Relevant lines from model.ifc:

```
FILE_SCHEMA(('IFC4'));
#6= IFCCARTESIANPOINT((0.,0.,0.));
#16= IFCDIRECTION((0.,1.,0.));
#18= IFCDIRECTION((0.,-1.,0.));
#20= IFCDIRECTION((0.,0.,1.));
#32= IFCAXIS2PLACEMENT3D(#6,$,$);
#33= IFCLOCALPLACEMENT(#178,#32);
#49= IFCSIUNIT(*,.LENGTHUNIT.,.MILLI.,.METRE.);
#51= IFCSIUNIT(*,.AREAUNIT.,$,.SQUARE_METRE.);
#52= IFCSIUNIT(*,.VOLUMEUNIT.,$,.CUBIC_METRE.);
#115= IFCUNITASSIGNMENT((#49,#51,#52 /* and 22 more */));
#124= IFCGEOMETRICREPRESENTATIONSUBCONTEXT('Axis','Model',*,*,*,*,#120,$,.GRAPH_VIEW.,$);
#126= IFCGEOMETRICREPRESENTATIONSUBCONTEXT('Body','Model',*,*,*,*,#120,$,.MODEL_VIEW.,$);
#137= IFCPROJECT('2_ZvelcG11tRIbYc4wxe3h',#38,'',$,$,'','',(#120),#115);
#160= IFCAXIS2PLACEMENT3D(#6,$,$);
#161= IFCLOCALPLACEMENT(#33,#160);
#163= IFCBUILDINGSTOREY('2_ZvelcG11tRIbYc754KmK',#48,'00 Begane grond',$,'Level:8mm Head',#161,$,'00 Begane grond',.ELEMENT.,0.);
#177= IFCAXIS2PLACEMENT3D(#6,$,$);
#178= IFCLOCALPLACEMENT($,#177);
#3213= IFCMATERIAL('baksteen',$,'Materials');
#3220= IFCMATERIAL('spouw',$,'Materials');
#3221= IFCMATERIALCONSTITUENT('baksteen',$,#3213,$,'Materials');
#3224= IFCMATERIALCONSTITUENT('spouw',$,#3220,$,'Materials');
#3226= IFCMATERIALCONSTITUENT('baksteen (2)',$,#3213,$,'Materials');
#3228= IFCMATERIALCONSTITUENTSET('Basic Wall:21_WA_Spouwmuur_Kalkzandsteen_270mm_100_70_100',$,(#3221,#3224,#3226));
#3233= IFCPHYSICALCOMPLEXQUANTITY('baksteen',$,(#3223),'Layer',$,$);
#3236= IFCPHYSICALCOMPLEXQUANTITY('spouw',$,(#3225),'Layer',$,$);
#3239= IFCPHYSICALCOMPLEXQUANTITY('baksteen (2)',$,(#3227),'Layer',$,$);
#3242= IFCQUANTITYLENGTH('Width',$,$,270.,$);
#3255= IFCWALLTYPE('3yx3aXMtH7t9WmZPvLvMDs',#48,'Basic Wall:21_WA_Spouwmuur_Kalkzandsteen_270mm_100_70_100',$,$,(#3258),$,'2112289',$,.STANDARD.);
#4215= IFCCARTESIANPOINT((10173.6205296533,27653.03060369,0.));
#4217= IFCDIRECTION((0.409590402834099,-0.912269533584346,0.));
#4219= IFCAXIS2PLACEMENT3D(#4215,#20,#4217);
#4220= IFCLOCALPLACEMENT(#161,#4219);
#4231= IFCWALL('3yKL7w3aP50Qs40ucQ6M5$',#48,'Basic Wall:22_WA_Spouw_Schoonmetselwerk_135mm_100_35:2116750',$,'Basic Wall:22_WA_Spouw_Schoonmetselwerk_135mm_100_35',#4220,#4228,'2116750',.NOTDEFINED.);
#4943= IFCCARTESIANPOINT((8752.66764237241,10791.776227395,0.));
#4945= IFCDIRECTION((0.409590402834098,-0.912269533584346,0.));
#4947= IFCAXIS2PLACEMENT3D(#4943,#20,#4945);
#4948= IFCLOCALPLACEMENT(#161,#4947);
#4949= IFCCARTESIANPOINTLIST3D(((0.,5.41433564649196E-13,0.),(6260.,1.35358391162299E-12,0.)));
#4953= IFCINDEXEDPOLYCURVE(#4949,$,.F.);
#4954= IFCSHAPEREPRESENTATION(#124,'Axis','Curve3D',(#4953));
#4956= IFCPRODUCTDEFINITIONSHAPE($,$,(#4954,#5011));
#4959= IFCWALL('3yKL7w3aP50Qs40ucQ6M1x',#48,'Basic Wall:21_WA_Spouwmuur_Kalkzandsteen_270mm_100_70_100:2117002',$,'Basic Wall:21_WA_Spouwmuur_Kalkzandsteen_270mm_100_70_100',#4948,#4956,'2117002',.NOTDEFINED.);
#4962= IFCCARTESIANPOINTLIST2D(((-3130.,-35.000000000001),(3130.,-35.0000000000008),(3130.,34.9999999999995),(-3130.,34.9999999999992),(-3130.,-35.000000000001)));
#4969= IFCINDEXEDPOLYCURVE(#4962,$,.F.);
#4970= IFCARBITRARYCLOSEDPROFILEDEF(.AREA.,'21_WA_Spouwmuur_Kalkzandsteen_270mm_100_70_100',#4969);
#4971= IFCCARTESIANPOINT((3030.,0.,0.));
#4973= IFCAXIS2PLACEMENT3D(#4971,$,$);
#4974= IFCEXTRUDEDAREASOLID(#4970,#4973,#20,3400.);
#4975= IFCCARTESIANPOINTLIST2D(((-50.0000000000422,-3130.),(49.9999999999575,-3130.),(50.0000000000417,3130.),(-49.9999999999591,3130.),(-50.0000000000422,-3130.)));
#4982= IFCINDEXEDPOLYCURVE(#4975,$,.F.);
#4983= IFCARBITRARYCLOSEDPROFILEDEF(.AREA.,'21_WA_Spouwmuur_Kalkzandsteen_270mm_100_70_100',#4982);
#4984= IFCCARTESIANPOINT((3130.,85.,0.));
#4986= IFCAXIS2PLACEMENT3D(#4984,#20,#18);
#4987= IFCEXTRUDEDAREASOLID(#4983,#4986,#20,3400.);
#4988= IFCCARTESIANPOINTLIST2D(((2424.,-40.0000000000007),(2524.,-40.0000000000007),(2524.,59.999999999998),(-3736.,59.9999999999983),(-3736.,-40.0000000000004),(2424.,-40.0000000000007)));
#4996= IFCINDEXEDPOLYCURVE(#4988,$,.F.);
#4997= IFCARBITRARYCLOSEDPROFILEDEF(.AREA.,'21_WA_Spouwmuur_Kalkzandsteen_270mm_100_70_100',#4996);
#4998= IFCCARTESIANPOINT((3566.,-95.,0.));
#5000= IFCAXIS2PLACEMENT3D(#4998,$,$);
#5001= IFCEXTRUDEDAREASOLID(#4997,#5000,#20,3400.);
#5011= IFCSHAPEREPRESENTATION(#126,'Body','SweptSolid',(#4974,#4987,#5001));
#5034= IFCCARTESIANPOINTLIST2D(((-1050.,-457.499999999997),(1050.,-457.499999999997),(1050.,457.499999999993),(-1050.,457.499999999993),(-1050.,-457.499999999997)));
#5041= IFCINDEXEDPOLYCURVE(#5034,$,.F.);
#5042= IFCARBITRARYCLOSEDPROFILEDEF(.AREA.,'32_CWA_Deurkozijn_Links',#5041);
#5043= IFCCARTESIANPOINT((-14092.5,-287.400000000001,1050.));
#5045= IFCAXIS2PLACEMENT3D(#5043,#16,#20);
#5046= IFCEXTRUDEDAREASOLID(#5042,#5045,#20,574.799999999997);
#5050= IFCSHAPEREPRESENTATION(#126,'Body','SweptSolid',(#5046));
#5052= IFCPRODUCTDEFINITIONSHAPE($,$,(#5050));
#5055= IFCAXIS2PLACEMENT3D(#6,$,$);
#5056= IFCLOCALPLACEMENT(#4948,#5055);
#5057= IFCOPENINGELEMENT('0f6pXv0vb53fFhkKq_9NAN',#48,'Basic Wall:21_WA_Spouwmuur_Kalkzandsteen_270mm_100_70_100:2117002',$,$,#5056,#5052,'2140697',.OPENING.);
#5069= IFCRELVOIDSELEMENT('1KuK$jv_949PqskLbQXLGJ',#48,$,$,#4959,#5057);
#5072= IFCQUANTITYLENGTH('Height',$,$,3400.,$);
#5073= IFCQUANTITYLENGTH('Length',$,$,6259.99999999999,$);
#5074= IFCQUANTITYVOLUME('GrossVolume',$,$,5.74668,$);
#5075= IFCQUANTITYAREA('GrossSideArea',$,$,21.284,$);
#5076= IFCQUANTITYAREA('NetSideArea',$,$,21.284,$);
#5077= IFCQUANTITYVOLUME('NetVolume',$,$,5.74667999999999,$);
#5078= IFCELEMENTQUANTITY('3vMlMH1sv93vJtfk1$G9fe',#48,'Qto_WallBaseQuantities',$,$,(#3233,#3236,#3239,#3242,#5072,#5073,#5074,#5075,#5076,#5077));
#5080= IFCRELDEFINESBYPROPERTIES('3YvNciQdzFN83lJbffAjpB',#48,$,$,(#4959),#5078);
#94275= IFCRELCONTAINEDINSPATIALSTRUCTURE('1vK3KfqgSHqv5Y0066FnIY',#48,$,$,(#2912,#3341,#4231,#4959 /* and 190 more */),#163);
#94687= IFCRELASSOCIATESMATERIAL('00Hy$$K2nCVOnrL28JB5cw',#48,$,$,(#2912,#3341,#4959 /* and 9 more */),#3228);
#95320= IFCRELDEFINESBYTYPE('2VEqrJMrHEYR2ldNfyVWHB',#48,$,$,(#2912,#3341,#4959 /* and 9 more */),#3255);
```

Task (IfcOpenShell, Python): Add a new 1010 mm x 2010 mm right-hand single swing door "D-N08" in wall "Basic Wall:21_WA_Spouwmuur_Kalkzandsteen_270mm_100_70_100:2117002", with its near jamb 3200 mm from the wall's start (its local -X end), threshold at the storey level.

```python
import numpy as np
import ifcopenshell
import ifcopenshell.api.feature
import ifcopenshell.api.geometry
import ifcopenshell.api.pset
import ifcopenshell.api.root
import ifcopenshell.api.spatial
import ifcopenshell.geom
import ifcopenshell.util.element
import ifcopenshell.util.placement
import ifcopenshell.util.representation
import ifcopenshell.util.shape
import ifcopenshell.util.unit

model = ifcopenshell.open("model.ifc")
unit_scale = ifcopenshell.util.unit.calculate_unit_scale(model)
area_scale = ifcopenshell.util.unit.calculate_unit_scale(model, "AREAUNIT")
volume_scale = ifcopenshell.util.unit.calculate_unit_scale(model, "VOLUMEUNIT")
settings = ifcopenshell.geom.settings()


def volume(element):
    """Net volume in cubic metres, openings subtracted."""
    shape = ifcopenshell.geom.create_shape(settings, element)
    return ifcopenshell.util.shape.get_volume(shape.geometry)


wall = model.by_guid("3yKL7w3aP50Qs40ucQ6M1x")
storey = ifcopenshell.util.element.get_container(wall, ifc_class="IfcBuildingStorey")
context = ifcopenshell.util.representation.get_context(model, "Model", "Body", "MODEL_VIEW")
before = volume(wall)

width, height, from_end, sill = 1.01, 2.01, 3.2, 0.0  # metres

# The wall runs along its own X axis, and the end named is its -X end.
wall_shape = ifcopenshell.geom.create_shape(settings, wall)
x, y, z = ifcopenshell.util.shape.get_vertices(wall_shape.geometry).T
start = x.min() + from_end
face, thickness = float(y.min()), float(y.max() - y.min())
wall_matrix = ifcopenshell.util.placement.get_local_placement(wall.ObjectPlacement)
level = ifcopenshell.util.placement.get_local_placement(storey.ObjectPlacement)[2, 3]


def in_wall(x, y):
    """Placement at x, y metres in the wall's axes, at sill height."""
    matrix = wall_matrix.copy()
    matrix[:, 3] = wall_matrix @ np.array([x / unit_scale, y / unit_scale, 0.0, 1.0])
    matrix[2, 3] = level + sill / unit_scale
    return matrix


# Opening: a box that overshoots both wall faces by 50 mm.
opening = ifcopenshell.api.root.create_entity(model, ifc_class="IfcOpeningElement", predefined_type="OPENING")
box = ifcopenshell.api.geometry.add_wall_representation(
    model, context=context, length=width, height=height, thickness=thickness + 0.1
)
ifcopenshell.api.geometry.assign_representation(model, product=opening, representation=box)
ifcopenshell.api.geometry.edit_object_placement(model, product=opening, matrix=in_wall(start, face - 0.05), is_si=False)
ifcopenshell.api.feature.add_feature(model, feature=opening, element=wall)

door = ifcopenshell.api.root.create_entity(model, ifc_class="IfcDoor", name="D-N08", predefined_type="DOOR")
door.OverallWidth, door.OverallHeight = width / unit_scale, height / unit_scale
door.OperationType = "SINGLE_SWING_RIGHT"
body = ifcopenshell.api.geometry.add_door_representation(
    model,
    context=context,
    overall_width=door.OverallWidth,
    overall_height=door.OverallHeight,
    operation_type="SINGLE_SWING_RIGHT",
    lining_properties={"LiningDepth": thickness / unit_scale, "ThresholdDepth": thickness / unit_scale},
)
ifcopenshell.api.geometry.assign_representation(model, product=door, representation=body)
ifcopenshell.api.spatial.assign_container(model, products=[door], relating_structure=storey)
ifcopenshell.api.feature.add_filling(model, opening=opening, element=door)

# The lining spans the wall, so the door starts at the wall face.
ifcopenshell.api.geometry.edit_object_placement(model, product=door, matrix=in_wall(start, face), is_si=False)

after = volume(wall)

# Update the wall's stored quantities.
qto = model.by_id(ifcopenshell.util.element.get_pset(wall, "Qto_WallBaseQuantities", should_inherit=False)["id"])
ifcopenshell.api.pset.edit_qto(model, qto=qto, properties={
    "NetSideArea": after / thickness / area_scale,
    "NetVolume": after / volume_scale,
})

print(f"wall volume {before:.3f} -> {after:.3f} m3")

model.write("model-out.ifc")
```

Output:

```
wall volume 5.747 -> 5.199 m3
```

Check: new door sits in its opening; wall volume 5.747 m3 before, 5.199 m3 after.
